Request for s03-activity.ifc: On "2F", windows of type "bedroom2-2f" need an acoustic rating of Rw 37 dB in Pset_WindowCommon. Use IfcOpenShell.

First a look at what the model holds.

```python
import ifcopenshell
import ifcopenshell.util.element

model = ifcopenshell.open("s03-activity.ifc")
print(model.schema)
storey = next(s for s in model.by_type("IfcBuildingStorey") if s.Name == "2F")
windows = [e for e in ifcopenshell.util.element.get_decomposition(storey) if e.is_a("IfcWindow")]
seen = {}
for e in windows:
    element_type = ifcopenshell.util.element.get_type(e)
    key = (element_type.Name if element_type != e and element_type else None, ifcopenshell.util.element.get_pset(e, "Pset_WindowCommon", "AcousticRating"))
    seen[key] = seen.get(key, 0) + 1
for (name, value), count in sorted(seen.items(), key=str):
    print(count, "x", name, "|", value)
```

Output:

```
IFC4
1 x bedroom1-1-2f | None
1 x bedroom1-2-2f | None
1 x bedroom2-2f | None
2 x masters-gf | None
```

```python
import ifcopenshell
import ifcopenshell.api.pset
import ifcopenshell.util.element

model = ifcopenshell.open("s03-activity.ifc")

storey = next(s for s in model.by_type("IfcBuildingStorey") if s.Name == "2F")
windows = [e for e in ifcopenshell.util.element.get_decomposition(storey) if e.is_a("IfcWindow")]

count = 0
for e in windows:
    element_type = ifcopenshell.util.element.get_type(e)
    if element_type in (None, e) or element_type.Name != "bedroom2-2f":
        continue
    # add_pset returns the element's existing set when there is one.
    pset = ifcopenshell.api.pset.add_pset(model, product=e, name="Pset_WindowCommon")
    ifcopenshell.api.pset.edit_pset(model, pset=pset, properties={"AcousticRating": "Rw 37 dB"})
    count += 1

print(count, "windows updated")

model.write("s03-activity_edited.ifc")
```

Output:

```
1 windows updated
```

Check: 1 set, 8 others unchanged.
